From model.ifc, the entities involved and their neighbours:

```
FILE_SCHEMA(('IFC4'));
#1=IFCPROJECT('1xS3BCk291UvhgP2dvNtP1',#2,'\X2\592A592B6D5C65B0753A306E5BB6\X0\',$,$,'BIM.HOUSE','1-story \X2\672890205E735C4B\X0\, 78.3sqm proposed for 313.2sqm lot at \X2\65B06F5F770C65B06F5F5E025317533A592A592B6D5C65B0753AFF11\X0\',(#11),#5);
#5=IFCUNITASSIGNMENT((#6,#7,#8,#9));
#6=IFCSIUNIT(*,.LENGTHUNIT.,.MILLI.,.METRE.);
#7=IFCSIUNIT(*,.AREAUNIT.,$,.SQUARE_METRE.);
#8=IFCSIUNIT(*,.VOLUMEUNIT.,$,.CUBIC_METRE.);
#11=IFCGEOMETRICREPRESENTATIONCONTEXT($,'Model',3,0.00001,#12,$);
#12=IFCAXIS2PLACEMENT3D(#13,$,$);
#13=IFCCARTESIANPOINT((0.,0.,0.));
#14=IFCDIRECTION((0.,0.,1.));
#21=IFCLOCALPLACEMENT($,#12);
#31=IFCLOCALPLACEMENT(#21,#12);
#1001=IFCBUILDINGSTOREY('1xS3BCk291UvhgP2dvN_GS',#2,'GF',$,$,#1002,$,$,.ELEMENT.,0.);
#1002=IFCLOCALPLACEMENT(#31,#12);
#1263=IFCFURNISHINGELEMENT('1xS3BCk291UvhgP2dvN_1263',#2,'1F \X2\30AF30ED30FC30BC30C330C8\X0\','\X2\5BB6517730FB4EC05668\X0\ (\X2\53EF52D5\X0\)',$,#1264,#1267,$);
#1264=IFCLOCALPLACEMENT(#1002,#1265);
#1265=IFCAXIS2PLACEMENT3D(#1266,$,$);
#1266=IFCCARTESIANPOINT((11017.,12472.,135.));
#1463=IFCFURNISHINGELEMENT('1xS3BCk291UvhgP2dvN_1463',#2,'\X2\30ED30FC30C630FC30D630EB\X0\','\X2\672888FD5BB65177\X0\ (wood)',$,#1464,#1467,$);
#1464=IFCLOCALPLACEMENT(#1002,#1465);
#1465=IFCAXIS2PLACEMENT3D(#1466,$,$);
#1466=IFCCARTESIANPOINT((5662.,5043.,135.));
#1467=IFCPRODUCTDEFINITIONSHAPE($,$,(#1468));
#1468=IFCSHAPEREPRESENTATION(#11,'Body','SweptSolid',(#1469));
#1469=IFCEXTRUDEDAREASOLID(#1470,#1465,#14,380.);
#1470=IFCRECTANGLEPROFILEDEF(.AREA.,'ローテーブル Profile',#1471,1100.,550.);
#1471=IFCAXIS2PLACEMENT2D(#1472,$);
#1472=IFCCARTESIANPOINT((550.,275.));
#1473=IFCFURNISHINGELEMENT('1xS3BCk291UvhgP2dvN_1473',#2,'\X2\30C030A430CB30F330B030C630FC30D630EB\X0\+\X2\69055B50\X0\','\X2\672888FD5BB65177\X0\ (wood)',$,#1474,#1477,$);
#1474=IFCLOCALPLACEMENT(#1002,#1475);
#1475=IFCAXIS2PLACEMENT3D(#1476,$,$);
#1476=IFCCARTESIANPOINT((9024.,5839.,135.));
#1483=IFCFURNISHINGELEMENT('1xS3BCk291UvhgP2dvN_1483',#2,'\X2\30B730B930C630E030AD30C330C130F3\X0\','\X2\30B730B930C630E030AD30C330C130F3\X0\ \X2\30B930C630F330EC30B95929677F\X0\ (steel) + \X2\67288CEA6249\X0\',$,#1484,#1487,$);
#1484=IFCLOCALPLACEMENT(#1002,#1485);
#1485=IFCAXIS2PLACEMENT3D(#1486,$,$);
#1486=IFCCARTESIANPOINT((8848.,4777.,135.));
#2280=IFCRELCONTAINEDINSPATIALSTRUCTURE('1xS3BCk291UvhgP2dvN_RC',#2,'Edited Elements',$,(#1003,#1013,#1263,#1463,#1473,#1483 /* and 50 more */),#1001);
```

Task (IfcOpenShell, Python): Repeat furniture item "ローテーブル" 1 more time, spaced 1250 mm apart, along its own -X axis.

```python
import ifcopenshell
import ifcopenshell.api.geometry
import ifcopenshell.api.root
import ifcopenshell.util.element
import ifcopenshell.util.placement
import ifcopenshell.util.unit

model = ifcopenshell.open("model.ifc")
unit_scale = ifcopenshell.util.unit.calculate_unit_scale(model)


def reuse_history(source, copy):
    """copy_class also copies each property set's owner history, people and application; keep the originals."""
    for rel in copy.IsDefinedBy:
        if rel.is_a("IfcRelDefinesByProperties") and (history := rel.RelatingPropertyDefinition.OwnerHistory):
            rel.RelatingPropertyDefinition.OwnerHistory = source.OwnerHistory
            ifcopenshell.util.element.remove_deep2(model, history)


source = model.by_id(1463)
base = ifcopenshell.util.placement.get_local_placement(source.ObjectPlacement)
step = -base[:3, 0] * 1.25 / unit_scale

for i in range(1, 2):
    copy = ifcopenshell.api.root.copy_class(model, product=source)
    copy.Representation = ifcopenshell.util.element.copy_deep(
        model, source.Representation, exclude=["IfcGeometricRepresentationContext", "IfcRepresentationMap"]
    )
    reuse_history(source, copy)
    matrix = base.copy()
    matrix[:3, 3] += i * step
    print("added at", matrix[:3, 3].round(3) + 0.0)
    ifcopenshell.api.geometry.edit_object_placement(model, product=copy, matrix=matrix, is_si=False)

model.write("model-out.ifc")
```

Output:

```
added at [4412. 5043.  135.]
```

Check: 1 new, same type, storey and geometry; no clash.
